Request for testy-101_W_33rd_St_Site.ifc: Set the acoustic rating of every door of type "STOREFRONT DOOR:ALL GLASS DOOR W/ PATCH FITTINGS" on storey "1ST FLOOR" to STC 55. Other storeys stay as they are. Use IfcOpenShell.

First a look at what the model holds.

```python
import ifcopenshell
import ifcopenshell.util.element

model = ifcopenshell.open("testy-101_W_33rd_St_Site.ifc")
print(model.schema)
storey = next(s for s in model.by_type("IfcBuildingStorey") if s.Name == "1ST FLOOR")
doors = [e for e in ifcopenshell.util.element.get_decomposition(storey) if e.is_a("IfcDoor")]
seen = {}
for e in doors:
    element_type = ifcopenshell.util.element.get_type(e)
    key = (element_type.Name if element_type != e and element_type else None, ifcopenshell.util.element.get_pset(e, "Pset_DoorCommon", "AcousticRating"))
    seen[key] = seen.get(key, 0) + 1
for (name, value), count in sorted(seen.items(), key=str):
    print(count, "x", name, "|", value)
```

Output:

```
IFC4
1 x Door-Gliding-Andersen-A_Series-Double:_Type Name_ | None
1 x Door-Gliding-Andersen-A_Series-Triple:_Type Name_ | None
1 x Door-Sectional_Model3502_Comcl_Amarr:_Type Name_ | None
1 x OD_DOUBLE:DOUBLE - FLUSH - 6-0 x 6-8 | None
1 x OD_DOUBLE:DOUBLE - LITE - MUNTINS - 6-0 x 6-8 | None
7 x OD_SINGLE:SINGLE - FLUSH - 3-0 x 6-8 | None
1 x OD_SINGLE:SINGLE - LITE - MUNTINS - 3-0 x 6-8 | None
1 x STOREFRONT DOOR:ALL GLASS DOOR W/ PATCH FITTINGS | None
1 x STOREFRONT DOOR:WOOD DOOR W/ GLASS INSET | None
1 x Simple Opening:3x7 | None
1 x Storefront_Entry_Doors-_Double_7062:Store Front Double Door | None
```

```python
import ifcopenshell
import ifcopenshell.api.pset
import ifcopenshell.util.element

model = ifcopenshell.open("testy-101_W_33rd_St_Site.ifc")

storey = next(s for s in model.by_type("IfcBuildingStorey") if s.Name == "1ST FLOOR")
doors = [e for e in ifcopenshell.util.element.get_decomposition(storey) if e.is_a("IfcDoor")]

count = 0
for e in doors:
    element_type = ifcopenshell.util.element.get_type(e)
    if element_type in (None, e) or element_type.Name != "STOREFRONT DOOR:ALL GLASS DOOR W/ PATCH FITTINGS":
        continue
    # add_pset returns the element's existing set when there is one.
    pset = ifcopenshell.api.pset.add_pset(model, product=e, name="Pset_DoorCommon")
    ifcopenshell.api.pset.edit_pset(model, pset=pset, properties={"AcousticRating": "STC 55"})
    count += 1

print(count, "doors updated")

model.write("testy-101_W_33rd_St_Site_edited.ifc")
```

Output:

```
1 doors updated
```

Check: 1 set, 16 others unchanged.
